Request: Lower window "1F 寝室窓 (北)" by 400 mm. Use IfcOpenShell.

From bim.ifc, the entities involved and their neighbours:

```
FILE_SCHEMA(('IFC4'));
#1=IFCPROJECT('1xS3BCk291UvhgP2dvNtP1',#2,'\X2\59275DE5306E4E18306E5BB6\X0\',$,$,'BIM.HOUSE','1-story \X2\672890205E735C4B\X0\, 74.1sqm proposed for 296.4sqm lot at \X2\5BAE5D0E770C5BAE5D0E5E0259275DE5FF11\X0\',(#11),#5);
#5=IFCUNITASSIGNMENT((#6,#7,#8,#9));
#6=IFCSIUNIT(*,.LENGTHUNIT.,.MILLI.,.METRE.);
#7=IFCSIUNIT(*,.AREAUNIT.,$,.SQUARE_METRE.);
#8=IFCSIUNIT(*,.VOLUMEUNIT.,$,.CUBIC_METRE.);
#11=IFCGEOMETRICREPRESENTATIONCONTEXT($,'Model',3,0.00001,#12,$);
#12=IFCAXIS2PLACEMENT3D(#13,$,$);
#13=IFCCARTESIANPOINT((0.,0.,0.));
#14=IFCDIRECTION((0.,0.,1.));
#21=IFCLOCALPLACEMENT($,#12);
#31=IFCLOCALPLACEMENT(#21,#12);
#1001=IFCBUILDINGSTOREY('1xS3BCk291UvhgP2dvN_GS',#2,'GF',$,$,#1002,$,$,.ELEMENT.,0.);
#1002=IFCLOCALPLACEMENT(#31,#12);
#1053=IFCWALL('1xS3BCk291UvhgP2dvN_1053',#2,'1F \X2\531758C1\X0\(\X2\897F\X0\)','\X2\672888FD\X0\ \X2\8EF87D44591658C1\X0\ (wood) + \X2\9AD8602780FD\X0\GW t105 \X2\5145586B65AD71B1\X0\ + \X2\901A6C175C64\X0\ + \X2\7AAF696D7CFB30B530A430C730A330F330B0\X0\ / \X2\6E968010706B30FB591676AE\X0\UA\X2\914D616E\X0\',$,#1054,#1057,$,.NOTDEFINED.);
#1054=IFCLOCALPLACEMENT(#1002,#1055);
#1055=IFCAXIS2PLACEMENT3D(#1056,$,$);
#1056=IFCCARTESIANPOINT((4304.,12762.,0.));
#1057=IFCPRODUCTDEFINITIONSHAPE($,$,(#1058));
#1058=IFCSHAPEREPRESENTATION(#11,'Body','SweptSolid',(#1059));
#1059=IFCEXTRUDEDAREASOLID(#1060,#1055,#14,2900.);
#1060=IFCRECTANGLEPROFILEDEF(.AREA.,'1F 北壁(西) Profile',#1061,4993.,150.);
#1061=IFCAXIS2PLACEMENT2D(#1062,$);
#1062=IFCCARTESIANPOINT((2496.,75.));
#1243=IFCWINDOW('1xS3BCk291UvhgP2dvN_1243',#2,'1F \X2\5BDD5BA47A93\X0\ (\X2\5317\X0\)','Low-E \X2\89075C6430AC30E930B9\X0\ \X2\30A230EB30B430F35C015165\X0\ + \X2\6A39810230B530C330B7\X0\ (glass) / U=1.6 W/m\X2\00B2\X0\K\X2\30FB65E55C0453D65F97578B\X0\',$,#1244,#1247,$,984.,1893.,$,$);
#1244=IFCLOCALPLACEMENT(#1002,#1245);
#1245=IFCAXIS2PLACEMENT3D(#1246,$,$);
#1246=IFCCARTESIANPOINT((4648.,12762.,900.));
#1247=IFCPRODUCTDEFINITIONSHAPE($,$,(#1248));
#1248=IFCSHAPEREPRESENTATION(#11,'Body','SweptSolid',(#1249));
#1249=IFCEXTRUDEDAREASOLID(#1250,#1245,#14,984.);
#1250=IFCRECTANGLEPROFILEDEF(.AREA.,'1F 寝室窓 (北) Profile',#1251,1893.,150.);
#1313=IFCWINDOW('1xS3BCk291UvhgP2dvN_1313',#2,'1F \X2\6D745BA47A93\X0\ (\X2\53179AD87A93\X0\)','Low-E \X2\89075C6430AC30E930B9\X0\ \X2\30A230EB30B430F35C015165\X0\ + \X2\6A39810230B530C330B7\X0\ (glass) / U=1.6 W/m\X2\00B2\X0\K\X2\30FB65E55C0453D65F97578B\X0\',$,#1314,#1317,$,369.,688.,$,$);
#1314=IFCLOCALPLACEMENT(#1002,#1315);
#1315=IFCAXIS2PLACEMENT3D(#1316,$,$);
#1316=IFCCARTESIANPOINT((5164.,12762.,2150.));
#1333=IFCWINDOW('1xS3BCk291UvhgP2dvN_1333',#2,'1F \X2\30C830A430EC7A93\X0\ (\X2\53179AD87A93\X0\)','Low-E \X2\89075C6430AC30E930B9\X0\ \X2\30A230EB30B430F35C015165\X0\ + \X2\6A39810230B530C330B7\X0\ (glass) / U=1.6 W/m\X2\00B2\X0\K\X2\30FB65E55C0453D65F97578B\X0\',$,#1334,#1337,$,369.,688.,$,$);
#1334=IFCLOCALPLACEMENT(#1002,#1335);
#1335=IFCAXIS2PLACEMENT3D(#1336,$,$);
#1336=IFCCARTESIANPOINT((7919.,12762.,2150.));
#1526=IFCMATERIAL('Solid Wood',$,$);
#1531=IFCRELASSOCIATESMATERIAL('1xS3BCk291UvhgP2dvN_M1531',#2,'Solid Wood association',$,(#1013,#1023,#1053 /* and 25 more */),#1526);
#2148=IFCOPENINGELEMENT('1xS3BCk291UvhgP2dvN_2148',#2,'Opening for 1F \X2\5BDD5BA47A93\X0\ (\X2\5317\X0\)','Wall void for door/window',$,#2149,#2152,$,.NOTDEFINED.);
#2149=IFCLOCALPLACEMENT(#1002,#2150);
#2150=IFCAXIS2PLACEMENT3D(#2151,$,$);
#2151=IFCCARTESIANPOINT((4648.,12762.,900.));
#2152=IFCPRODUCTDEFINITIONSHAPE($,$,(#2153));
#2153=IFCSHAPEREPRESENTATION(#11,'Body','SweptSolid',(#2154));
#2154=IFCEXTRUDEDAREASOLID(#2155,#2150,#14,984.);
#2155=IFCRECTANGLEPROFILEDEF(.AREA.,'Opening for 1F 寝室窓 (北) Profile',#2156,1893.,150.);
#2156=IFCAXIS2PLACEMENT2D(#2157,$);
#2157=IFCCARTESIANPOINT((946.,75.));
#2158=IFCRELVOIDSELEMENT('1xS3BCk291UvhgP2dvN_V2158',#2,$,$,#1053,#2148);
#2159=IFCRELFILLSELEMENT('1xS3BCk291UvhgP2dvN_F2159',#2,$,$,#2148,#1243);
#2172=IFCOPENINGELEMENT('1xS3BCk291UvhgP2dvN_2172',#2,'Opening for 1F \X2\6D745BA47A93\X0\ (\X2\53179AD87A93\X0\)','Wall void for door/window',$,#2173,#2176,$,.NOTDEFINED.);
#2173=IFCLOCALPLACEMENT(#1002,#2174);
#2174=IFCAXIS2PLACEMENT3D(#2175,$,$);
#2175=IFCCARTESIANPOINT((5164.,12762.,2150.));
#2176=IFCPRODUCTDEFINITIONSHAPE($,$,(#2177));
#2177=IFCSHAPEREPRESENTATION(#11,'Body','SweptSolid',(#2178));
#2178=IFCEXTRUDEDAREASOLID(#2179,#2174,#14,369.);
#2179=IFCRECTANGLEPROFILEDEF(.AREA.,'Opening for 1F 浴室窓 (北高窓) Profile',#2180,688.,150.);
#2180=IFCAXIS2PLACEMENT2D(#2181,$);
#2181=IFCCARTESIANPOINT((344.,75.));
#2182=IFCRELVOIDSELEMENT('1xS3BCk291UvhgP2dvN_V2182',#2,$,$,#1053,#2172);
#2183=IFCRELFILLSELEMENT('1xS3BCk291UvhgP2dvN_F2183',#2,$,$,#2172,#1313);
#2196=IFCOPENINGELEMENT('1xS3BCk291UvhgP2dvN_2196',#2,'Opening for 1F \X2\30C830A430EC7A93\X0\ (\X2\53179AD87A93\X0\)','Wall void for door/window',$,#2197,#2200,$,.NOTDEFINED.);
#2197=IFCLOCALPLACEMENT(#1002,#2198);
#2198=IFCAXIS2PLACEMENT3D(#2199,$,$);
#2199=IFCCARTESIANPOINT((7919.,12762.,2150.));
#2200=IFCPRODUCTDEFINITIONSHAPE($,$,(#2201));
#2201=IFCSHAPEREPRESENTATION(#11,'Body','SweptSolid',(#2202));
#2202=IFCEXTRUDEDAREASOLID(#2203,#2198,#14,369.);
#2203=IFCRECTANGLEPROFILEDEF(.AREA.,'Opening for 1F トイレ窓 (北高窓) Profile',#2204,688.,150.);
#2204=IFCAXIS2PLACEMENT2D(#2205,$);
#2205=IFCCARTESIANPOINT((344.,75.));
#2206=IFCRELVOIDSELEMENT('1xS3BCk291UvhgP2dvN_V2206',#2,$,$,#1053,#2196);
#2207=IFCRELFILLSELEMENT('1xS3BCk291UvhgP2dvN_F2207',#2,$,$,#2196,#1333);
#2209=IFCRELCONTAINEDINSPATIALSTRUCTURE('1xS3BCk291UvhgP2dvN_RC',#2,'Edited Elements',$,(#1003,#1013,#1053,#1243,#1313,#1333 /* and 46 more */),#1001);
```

```python
import numpy as np
import ifcopenshell
import ifcopenshell.api.geometry
import ifcopenshell.util.placement
import ifcopenshell.util.unit

model = ifcopenshell.open("bim.ifc")
unit_scale = ifcopenshell.util.unit.calculate_unit_scale(model)

window = model.by_guid("1xS3BCk291UvhgP2dvN_1243")
opening = window.FillsVoids[0].RelatingOpeningElement
dz = -400.0

shift = np.array([0.0, 0.0, dz])
# The window is not placed relative to its opening, so move both.
for product in (opening, window):
    matrix = ifcopenshell.util.placement.get_local_placement(product.ObjectPlacement)
    matrix[:3, 3] += shift
    ifcopenshell.api.geometry.edit_object_placement(model, product=product, matrix=matrix, is_si=False)

print(f"moved by {dz * unit_scale:+.3f} m")

model.write("bim_rev.ifc")
```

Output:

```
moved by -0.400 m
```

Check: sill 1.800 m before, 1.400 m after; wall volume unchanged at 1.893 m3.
